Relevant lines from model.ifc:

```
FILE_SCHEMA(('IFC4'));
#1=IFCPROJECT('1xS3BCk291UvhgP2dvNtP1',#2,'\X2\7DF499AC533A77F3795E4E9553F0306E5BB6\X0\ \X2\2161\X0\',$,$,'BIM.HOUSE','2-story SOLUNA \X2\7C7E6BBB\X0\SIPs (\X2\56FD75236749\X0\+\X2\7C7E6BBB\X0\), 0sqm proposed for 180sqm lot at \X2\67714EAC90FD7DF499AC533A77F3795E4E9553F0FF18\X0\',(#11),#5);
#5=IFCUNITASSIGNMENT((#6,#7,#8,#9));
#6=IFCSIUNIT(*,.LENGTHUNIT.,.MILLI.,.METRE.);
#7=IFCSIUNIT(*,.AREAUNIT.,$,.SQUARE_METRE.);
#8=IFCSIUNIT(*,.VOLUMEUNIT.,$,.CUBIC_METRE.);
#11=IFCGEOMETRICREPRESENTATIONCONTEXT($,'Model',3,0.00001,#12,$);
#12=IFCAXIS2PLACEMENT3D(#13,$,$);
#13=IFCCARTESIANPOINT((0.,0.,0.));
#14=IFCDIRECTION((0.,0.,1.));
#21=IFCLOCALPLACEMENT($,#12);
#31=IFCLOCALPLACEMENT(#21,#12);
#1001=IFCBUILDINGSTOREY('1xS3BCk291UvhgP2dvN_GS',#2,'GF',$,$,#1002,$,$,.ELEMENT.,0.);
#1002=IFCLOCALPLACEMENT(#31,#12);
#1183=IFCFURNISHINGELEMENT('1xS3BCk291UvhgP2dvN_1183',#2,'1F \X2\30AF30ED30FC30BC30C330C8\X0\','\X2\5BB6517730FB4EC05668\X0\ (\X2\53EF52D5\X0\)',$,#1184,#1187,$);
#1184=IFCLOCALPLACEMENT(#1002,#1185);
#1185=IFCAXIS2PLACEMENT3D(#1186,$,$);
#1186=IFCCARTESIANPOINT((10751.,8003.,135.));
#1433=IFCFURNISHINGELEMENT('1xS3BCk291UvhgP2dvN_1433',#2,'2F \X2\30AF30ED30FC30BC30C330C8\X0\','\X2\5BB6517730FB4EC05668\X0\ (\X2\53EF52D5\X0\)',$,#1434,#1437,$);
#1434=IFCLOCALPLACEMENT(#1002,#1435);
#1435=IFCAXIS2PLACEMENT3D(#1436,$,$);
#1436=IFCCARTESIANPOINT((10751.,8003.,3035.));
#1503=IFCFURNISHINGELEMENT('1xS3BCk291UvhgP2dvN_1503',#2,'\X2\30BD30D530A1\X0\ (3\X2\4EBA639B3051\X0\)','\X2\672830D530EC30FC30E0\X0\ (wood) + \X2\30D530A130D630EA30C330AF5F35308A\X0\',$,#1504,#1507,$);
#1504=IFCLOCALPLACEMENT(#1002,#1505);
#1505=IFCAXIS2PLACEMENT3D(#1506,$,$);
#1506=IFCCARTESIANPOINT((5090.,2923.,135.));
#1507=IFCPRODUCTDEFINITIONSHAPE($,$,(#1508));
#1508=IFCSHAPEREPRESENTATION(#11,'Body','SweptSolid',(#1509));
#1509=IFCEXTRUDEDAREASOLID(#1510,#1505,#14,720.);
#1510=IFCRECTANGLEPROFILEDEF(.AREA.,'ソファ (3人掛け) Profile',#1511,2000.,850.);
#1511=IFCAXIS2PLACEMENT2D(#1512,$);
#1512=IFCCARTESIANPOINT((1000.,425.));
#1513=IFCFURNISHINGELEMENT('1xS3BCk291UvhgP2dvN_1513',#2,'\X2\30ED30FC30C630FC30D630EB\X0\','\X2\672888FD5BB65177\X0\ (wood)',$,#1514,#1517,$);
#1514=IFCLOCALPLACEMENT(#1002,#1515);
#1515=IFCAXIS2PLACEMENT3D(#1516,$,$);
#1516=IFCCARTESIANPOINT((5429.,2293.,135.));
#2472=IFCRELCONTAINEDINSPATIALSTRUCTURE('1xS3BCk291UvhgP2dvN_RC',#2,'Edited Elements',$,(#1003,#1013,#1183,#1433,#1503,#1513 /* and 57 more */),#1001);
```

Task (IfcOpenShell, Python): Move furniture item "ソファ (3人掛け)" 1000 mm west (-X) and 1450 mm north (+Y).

```python
import ifcopenshell
import ifcopenshell.api.geometry
import ifcopenshell.util.placement
import ifcopenshell.util.unit

model = ifcopenshell.open("model.ifc")
unit_scale = ifcopenshell.util.unit.calculate_unit_scale(model)

item = model.by_id(1503)
matrix = ifcopenshell.util.placement.get_local_placement(item.ObjectPlacement)
matrix[0, 3] -= 1 / unit_scale
matrix[1, 3] += 1.45 / unit_scale
ifcopenshell.api.geometry.edit_object_placement(model, product=item, matrix=matrix, is_si=False)

print(ifcopenshell.util.placement.get_local_placement(item.ObjectPlacement).round(3) + 0.0)

model.write("model_edited.ifc")
```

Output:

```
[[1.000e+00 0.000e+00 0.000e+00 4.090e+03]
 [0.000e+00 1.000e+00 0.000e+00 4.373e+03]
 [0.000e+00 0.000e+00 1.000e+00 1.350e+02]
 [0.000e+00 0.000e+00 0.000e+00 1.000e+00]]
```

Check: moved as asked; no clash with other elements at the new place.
